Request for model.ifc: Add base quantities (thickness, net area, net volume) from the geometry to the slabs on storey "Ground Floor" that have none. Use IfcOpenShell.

First a look at what the model holds.

```python
import ifcopenshell
import ifcopenshell.util.element
import ifcopenshell.util.unit

model = ifcopenshell.open("model.ifc")
print(model.schema)
for unit_type in ("LENGTHUNIT", "AREAUNIT", "VOLUMEUNIT"):
    print(unit_type, ifcopenshell.util.unit.calculate_unit_scale(model, unit_type))
storey = next(s for s in model.by_type("IfcBuildingStorey") if s.Name == "Ground Floor")
slabs = [e for e in ifcopenshell.util.element.get_decomposition(storey) if e.is_a("IfcSlab")]
for e in sorted(slabs, key=lambda e: e.id()):
    print(e.id(), e.is_a(), e.Name, list(ifcopenshell.util.element.get_psets(e, qtos_only=True)), sep=" | ")
```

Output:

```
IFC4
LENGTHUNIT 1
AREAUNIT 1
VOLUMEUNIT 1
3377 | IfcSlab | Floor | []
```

```python
import ifcopenshell
import ifcopenshell.api.pset
import ifcopenshell.geom
import ifcopenshell.util.element
import ifcopenshell.util.shape
import ifcopenshell.util.unit

model = ifcopenshell.open("model.ifc")
unit_scale = ifcopenshell.util.unit.calculate_unit_scale(model)
area_scale = ifcopenshell.util.unit.calculate_unit_scale(model, "AREAUNIT")
volume_scale = ifcopenshell.util.unit.calculate_unit_scale(model, "VOLUMEUNIT")
settings = ifcopenshell.geom.settings()

storey = next(s for s in model.by_type("IfcBuildingStorey") if s.Name == "Ground Floor")
slabs = [e for e in ifcopenshell.util.element.get_decomposition(storey) if e.is_a("IfcSlab")]

for e in sorted(slabs, key=lambda e: e.id()):
    if ifcopenshell.util.element.get_psets(e, qtos_only=True, should_inherit=False):
        continue
    # Geometry comes back in metres, in the element's own axes.
    shape = ifcopenshell.geom.create_shape(settings, e)
    values = {
        "Width": ifcopenshell.util.shape.get_z(shape.geometry) / unit_scale,
        "NetArea": ifcopenshell.util.shape.get_footprint_area(shape.geometry) / area_scale,
        "NetVolume": ifcopenshell.util.shape.get_volume(shape.geometry) / volume_scale,
    }
    qto = ifcopenshell.api.pset.add_qto(model, product=e, name="Qto_SlabBaseQuantities")
    ifcopenshell.api.pset.edit_qto(model, qto=qto, properties=values)
    print(e.id(), {k: round(v, 3) for k, v in values.items()})

model.write("model_v2.ifc")
```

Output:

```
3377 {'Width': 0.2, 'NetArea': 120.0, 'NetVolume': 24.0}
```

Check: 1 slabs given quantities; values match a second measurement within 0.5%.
